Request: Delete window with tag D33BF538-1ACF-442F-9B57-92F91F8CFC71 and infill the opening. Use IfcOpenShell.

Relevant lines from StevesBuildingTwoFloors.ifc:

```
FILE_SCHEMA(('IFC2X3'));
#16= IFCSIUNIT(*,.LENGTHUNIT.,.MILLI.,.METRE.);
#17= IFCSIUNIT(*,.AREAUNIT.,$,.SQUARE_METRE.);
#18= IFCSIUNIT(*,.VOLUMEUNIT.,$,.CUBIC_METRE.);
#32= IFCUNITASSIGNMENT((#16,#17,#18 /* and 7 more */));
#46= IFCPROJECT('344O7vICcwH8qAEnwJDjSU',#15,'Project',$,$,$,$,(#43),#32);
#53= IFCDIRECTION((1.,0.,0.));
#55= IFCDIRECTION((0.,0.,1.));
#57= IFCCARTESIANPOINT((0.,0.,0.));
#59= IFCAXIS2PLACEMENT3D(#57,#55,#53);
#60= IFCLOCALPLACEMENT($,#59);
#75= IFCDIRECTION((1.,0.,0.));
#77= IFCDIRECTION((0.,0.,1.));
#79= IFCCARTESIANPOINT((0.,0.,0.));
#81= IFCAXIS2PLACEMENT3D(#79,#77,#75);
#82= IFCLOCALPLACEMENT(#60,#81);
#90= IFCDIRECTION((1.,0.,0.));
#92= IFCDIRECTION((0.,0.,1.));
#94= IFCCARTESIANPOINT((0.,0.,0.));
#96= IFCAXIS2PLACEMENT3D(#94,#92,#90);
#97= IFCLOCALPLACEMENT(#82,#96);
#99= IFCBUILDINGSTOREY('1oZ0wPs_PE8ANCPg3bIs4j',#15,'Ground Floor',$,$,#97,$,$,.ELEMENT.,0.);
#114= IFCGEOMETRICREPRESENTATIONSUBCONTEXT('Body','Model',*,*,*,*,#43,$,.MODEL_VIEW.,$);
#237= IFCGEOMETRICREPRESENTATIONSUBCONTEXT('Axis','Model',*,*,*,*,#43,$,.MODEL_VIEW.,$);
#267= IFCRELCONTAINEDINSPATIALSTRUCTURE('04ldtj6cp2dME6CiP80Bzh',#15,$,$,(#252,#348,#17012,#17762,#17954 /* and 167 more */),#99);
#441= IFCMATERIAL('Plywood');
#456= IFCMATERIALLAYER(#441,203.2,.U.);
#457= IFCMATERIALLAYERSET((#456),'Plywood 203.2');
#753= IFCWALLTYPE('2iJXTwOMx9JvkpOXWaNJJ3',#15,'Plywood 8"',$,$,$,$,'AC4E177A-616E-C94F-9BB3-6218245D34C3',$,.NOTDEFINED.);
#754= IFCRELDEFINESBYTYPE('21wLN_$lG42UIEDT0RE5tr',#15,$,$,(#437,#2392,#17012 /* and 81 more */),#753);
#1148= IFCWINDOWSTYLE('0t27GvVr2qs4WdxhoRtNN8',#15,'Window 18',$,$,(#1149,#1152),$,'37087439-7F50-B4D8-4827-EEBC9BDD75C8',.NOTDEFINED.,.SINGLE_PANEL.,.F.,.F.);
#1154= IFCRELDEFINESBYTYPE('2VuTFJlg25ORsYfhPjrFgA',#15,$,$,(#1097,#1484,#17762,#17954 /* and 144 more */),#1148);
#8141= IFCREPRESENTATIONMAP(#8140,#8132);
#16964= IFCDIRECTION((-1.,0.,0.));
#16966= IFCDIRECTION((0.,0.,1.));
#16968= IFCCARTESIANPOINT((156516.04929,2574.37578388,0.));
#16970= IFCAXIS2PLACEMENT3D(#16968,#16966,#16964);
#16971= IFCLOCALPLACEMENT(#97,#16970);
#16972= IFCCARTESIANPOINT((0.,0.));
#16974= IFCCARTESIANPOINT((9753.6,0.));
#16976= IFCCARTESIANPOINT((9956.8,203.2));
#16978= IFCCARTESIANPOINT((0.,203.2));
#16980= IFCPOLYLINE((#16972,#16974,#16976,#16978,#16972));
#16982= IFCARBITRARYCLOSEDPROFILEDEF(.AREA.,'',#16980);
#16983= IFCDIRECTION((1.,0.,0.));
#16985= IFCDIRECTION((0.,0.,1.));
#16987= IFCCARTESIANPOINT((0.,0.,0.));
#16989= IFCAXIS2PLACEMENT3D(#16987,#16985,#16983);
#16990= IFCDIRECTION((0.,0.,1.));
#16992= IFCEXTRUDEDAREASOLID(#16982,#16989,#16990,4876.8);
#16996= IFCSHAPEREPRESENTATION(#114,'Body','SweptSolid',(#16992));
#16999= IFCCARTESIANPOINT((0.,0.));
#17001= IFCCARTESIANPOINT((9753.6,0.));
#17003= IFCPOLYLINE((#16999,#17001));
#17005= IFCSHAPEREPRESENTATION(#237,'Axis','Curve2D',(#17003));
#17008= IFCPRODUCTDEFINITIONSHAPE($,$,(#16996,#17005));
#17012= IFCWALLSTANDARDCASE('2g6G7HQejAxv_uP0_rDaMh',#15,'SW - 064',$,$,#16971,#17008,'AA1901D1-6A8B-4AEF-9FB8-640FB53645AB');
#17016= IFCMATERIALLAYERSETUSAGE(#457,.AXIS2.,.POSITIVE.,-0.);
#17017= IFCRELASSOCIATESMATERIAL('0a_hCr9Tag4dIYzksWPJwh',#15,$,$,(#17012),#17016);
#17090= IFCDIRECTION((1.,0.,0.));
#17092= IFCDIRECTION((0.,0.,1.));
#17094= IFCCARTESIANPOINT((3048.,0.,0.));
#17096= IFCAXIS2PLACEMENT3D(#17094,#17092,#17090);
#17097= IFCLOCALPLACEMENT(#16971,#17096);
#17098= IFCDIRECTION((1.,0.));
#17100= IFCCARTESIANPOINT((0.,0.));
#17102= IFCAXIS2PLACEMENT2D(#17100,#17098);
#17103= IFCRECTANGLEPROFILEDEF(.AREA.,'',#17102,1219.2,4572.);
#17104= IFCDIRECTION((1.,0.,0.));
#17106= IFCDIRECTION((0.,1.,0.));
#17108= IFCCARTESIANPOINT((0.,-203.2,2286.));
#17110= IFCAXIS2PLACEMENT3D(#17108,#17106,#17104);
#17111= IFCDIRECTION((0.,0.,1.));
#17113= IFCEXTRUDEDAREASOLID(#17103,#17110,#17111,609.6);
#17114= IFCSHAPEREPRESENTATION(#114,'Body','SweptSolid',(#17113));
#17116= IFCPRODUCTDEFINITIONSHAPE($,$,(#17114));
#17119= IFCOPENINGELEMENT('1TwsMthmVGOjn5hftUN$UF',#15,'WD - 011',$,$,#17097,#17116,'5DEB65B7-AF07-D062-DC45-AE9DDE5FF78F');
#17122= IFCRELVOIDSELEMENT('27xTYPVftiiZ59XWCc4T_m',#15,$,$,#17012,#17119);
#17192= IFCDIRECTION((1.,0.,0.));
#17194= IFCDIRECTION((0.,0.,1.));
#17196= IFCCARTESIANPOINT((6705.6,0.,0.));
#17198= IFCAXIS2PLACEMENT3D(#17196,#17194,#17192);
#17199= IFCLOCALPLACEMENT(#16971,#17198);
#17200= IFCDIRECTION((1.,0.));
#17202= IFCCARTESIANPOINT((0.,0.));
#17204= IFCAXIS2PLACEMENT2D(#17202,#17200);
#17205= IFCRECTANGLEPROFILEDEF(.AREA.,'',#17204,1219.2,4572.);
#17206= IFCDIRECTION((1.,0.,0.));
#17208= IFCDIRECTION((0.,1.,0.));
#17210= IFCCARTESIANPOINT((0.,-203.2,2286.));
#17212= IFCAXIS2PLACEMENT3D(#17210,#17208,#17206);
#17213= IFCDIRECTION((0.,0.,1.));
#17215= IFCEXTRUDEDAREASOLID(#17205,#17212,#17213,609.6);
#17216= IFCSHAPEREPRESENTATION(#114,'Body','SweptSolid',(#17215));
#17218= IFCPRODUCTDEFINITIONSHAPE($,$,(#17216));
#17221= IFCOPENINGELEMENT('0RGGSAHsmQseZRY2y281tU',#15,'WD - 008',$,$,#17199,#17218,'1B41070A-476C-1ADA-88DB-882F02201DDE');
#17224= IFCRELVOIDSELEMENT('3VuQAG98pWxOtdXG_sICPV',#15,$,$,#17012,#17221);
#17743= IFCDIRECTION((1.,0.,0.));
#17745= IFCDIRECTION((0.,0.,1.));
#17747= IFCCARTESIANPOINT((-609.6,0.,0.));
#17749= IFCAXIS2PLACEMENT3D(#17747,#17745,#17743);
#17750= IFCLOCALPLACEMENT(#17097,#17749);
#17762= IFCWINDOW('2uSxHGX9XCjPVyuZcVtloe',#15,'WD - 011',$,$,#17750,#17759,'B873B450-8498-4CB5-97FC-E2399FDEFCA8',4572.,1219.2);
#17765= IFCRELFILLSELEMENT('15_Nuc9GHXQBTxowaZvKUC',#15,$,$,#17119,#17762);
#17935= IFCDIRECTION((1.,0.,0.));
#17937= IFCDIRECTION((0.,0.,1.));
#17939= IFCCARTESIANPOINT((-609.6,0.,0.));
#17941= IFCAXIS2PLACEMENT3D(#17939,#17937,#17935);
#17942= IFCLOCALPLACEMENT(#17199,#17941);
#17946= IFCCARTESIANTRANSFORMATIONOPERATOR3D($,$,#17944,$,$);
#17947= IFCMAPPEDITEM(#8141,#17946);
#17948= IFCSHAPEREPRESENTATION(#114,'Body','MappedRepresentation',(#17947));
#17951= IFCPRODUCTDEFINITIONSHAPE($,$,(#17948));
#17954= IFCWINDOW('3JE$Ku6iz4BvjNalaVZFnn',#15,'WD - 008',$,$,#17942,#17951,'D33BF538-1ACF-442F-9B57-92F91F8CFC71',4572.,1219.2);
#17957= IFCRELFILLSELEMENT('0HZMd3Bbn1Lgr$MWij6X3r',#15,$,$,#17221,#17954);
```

```python
import ifcopenshell
import ifcopenshell.api.feature
import ifcopenshell.api.root
import ifcopenshell.geom
import ifcopenshell.util.shape

model = ifcopenshell.open("StevesBuildingTwoFloors.ifc")
settings = ifcopenshell.geom.settings()


def volume(element):
    """Net volume in cubic metres, openings subtracted."""
    shape = ifcopenshell.geom.create_shape(settings, element)
    return ifcopenshell.util.shape.get_volume(shape.geometry)


window = model.by_guid("3JE$Ku6iz4BvjNalaVZFnn")
opening = window.FillsVoids[0].RelatingOpeningElement
wall = opening.VoidsElements[0].RelatingBuildingElement
before = volume(wall)

ifcopenshell.api.root.remove_product(model, product=window)
ifcopenshell.api.feature.remove_feature(model, feature=opening)

after = volume(wall)

print(f"wall volume {before:.3f} -> {after:.3f} m3")

model.write("StevesBuildingTwoFloors_v2.ifc")
```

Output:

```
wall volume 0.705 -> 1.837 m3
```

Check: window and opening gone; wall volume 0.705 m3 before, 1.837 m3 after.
